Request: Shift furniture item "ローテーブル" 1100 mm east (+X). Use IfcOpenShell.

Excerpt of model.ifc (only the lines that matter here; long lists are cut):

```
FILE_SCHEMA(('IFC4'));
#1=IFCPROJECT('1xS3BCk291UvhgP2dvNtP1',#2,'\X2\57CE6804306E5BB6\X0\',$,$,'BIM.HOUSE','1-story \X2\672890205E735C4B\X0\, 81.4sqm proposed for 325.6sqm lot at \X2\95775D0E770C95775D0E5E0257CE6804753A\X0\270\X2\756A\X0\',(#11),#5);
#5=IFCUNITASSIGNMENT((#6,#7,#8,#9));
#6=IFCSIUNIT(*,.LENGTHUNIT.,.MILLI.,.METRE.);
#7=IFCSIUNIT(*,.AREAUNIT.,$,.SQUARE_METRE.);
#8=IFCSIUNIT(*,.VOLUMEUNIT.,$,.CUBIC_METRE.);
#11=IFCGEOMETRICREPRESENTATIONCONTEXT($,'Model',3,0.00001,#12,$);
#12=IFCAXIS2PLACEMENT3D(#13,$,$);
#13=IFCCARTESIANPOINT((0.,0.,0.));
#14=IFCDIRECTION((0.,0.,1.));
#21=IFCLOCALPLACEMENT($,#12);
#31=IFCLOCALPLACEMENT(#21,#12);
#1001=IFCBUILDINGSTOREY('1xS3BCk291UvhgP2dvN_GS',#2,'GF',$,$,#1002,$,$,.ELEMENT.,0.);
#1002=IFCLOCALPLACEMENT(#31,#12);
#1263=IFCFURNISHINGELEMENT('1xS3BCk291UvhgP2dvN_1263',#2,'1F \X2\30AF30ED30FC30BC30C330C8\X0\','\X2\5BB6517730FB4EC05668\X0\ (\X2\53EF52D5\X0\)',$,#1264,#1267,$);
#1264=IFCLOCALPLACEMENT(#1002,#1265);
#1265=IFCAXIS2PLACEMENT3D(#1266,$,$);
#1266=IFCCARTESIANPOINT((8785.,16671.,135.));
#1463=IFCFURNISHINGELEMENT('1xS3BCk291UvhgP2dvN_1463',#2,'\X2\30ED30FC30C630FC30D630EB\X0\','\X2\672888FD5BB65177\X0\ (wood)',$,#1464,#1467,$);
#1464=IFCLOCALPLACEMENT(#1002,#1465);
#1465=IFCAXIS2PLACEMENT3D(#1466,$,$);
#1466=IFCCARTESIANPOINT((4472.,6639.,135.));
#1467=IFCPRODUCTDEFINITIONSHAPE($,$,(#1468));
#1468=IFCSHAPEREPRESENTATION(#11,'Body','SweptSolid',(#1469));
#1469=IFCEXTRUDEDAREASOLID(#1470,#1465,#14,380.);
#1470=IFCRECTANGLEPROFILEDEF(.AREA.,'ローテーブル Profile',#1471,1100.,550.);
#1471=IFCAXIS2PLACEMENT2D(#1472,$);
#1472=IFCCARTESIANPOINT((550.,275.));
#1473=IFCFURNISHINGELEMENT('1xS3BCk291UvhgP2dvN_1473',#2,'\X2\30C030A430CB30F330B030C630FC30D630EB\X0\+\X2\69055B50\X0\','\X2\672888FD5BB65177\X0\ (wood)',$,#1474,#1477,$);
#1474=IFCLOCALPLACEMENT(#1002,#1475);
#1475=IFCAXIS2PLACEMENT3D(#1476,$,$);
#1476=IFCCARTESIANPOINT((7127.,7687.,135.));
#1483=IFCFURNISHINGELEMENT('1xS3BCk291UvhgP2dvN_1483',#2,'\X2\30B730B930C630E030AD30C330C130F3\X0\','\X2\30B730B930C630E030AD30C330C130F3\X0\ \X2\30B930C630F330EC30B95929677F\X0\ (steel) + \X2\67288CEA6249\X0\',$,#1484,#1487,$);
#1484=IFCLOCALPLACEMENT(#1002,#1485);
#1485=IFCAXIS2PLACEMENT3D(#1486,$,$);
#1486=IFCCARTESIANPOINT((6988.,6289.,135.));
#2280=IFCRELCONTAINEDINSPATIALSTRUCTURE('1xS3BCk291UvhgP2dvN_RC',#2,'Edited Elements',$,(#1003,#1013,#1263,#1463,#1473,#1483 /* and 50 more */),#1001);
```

```python
import ifcopenshell
import ifcopenshell.api.geometry
import ifcopenshell.util.placement

model = ifcopenshell.open("model.ifc")

item = model.by_id(1463)
matrix = ifcopenshell.util.placement.get_local_placement(item.ObjectPlacement)
matrix[0, 3] += 1100.0
ifcopenshell.api.geometry.edit_object_placement(model, product=item, matrix=matrix, is_si=False)

print(ifcopenshell.util.placement.get_local_placement(item.ObjectPlacement).round(3) + 0.0)

model.write("model_rev.ifc")
```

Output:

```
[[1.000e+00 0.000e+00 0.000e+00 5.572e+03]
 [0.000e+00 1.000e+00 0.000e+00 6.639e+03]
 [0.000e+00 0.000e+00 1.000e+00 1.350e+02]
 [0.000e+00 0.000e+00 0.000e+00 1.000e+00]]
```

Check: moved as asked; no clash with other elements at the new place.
